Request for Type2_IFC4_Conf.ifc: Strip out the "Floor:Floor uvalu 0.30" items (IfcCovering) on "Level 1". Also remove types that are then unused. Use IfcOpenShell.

First a look at what the model holds.

```python
import ifcopenshell
import ifcopenshell.util.element

model = ifcopenshell.open("Type2_IFC4_Conf.ifc")
print(model.schema)
storey = next(s for s in model.by_type("IfcBuildingStorey") if s.Name == "Level 1")
coverings = [e for e in ifcopenshell.util.element.get_decomposition(storey) if e.is_a("IfcCovering")]
seen = {}
for e in coverings:
    element_type = ifcopenshell.util.element.get_type(e)
    name = element_type.Name if element_type not in (None, e) else None
    seen[name] = seen.get(name, 0) + 1
for name, count in sorted(seen.items(), key=str):
    print(count, "x", name)
```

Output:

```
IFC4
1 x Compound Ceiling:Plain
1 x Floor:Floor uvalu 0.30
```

```python
import ifcopenshell
import ifcopenshell.api.root
import ifcopenshell.util.element

model = ifcopenshell.open("Type2_IFC4_Conf.ifc")

storey = next(s for s in model.by_type("IfcBuildingStorey") if s.Name == "Level 1")
coverings = [e for e in ifcopenshell.util.element.get_decomposition(storey) if e.is_a("IfcCovering")]
targets = [e for e in coverings if (t := ifcopenshell.util.element.get_type(e)) not in (None, e) and t.Name == "Floor:Floor uvalu 0.30"]
types = {ifcopenshell.util.element.get_type(e) for e in targets} - {None, *targets}

for e in targets:
    ifcopenshell.api.root.remove_product(model, product=e)
print(len(targets), "removed")

unused = [t for t in types if not ifcopenshell.util.element.get_types(t)]
for t in unused:
    ifcopenshell.api.root.remove_product(model, product=t)
print(len(unused), "unused types removed")

model.write("Type2_IFC4_Conf_updated.ifc")
```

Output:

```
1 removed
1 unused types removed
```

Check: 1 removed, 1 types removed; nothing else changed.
